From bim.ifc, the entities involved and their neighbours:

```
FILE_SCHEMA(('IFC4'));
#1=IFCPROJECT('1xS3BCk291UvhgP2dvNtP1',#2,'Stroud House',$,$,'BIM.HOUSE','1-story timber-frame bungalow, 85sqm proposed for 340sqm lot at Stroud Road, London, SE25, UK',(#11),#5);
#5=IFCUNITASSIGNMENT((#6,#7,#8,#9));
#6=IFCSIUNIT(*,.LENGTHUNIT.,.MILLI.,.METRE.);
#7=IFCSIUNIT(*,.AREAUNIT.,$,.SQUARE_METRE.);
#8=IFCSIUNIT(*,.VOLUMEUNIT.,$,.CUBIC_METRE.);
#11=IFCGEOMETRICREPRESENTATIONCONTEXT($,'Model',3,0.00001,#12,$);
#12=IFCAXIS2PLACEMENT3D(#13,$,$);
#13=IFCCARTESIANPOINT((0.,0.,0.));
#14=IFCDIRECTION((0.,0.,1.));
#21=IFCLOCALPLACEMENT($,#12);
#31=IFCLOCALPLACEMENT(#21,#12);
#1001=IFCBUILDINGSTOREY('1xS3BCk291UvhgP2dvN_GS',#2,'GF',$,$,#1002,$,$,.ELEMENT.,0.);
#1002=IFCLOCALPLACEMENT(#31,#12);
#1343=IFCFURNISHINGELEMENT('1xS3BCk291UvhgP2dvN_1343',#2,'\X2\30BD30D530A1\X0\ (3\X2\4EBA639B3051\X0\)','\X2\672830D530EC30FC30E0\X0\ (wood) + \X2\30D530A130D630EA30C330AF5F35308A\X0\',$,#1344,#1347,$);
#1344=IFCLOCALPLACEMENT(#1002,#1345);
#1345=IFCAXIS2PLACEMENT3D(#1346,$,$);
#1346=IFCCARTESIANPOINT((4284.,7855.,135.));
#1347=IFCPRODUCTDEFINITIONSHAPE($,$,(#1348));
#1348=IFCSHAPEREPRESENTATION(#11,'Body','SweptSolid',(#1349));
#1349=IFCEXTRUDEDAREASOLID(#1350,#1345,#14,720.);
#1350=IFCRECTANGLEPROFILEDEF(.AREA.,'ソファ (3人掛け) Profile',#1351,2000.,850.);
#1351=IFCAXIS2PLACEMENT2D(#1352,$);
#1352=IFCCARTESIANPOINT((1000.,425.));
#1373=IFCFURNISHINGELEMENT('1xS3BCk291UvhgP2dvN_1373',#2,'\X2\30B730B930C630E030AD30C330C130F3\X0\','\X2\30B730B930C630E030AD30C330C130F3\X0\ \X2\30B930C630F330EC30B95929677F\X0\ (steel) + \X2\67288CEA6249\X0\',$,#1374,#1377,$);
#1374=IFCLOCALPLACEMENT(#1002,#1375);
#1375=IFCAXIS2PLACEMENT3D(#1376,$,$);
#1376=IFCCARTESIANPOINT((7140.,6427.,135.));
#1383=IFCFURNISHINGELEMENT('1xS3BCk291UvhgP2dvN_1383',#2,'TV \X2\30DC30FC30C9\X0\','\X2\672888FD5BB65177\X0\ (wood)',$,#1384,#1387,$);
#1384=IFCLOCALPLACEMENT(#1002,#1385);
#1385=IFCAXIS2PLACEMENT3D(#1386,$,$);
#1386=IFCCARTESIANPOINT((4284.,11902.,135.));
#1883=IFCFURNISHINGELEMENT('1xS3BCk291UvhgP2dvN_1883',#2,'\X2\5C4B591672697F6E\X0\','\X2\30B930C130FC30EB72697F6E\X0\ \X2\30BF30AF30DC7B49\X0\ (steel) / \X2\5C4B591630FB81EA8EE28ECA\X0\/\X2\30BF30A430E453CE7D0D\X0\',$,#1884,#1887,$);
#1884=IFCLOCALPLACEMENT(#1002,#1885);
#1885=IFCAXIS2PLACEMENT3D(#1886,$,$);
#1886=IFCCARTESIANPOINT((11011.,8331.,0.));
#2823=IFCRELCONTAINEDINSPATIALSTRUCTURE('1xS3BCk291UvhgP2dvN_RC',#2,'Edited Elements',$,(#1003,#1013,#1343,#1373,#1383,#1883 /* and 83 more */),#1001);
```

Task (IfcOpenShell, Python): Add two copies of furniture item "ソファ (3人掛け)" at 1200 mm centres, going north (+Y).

```python
import numpy as np
import ifcopenshell
import ifcopenshell.api.geometry
import ifcopenshell.api.root
import ifcopenshell.util.element
import ifcopenshell.util.placement
import ifcopenshell.util.unit

model = ifcopenshell.open("bim.ifc")
unit_scale = ifcopenshell.util.unit.calculate_unit_scale(model)


def reuse_history(source, copy):
    """copy_class also copies each property set's owner history, people and application; keep the originals."""
    for rel in copy.IsDefinedBy:
        if rel.is_a("IfcRelDefinesByProperties") and (history := rel.RelatingPropertyDefinition.OwnerHistory):
            rel.RelatingPropertyDefinition.OwnerHistory = source.OwnerHistory
            ifcopenshell.util.element.remove_deep2(model, history)


source = model.by_id(1343)
base = ifcopenshell.util.placement.get_local_placement(source.ObjectPlacement)
step = np.array([0.0, 1.0, 0.0]) * 1.2 / unit_scale

for i in range(1, 3):
    copy = ifcopenshell.api.root.copy_class(model, product=source)
    copy.Representation = ifcopenshell.util.element.copy_deep(
        model, source.Representation, exclude=["IfcGeometricRepresentationContext", "IfcRepresentationMap"]
    )
    reuse_history(source, copy)
    matrix = base.copy()
    matrix[:3, 3] += i * step
    print("added at", matrix[:3, 3].round(3) + 0.0)
    ifcopenshell.api.geometry.edit_object_placement(model, product=copy, matrix=matrix, is_si=False)

model.write("bim_v2.ifc")
```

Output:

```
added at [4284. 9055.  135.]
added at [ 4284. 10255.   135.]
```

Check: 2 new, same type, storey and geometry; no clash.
